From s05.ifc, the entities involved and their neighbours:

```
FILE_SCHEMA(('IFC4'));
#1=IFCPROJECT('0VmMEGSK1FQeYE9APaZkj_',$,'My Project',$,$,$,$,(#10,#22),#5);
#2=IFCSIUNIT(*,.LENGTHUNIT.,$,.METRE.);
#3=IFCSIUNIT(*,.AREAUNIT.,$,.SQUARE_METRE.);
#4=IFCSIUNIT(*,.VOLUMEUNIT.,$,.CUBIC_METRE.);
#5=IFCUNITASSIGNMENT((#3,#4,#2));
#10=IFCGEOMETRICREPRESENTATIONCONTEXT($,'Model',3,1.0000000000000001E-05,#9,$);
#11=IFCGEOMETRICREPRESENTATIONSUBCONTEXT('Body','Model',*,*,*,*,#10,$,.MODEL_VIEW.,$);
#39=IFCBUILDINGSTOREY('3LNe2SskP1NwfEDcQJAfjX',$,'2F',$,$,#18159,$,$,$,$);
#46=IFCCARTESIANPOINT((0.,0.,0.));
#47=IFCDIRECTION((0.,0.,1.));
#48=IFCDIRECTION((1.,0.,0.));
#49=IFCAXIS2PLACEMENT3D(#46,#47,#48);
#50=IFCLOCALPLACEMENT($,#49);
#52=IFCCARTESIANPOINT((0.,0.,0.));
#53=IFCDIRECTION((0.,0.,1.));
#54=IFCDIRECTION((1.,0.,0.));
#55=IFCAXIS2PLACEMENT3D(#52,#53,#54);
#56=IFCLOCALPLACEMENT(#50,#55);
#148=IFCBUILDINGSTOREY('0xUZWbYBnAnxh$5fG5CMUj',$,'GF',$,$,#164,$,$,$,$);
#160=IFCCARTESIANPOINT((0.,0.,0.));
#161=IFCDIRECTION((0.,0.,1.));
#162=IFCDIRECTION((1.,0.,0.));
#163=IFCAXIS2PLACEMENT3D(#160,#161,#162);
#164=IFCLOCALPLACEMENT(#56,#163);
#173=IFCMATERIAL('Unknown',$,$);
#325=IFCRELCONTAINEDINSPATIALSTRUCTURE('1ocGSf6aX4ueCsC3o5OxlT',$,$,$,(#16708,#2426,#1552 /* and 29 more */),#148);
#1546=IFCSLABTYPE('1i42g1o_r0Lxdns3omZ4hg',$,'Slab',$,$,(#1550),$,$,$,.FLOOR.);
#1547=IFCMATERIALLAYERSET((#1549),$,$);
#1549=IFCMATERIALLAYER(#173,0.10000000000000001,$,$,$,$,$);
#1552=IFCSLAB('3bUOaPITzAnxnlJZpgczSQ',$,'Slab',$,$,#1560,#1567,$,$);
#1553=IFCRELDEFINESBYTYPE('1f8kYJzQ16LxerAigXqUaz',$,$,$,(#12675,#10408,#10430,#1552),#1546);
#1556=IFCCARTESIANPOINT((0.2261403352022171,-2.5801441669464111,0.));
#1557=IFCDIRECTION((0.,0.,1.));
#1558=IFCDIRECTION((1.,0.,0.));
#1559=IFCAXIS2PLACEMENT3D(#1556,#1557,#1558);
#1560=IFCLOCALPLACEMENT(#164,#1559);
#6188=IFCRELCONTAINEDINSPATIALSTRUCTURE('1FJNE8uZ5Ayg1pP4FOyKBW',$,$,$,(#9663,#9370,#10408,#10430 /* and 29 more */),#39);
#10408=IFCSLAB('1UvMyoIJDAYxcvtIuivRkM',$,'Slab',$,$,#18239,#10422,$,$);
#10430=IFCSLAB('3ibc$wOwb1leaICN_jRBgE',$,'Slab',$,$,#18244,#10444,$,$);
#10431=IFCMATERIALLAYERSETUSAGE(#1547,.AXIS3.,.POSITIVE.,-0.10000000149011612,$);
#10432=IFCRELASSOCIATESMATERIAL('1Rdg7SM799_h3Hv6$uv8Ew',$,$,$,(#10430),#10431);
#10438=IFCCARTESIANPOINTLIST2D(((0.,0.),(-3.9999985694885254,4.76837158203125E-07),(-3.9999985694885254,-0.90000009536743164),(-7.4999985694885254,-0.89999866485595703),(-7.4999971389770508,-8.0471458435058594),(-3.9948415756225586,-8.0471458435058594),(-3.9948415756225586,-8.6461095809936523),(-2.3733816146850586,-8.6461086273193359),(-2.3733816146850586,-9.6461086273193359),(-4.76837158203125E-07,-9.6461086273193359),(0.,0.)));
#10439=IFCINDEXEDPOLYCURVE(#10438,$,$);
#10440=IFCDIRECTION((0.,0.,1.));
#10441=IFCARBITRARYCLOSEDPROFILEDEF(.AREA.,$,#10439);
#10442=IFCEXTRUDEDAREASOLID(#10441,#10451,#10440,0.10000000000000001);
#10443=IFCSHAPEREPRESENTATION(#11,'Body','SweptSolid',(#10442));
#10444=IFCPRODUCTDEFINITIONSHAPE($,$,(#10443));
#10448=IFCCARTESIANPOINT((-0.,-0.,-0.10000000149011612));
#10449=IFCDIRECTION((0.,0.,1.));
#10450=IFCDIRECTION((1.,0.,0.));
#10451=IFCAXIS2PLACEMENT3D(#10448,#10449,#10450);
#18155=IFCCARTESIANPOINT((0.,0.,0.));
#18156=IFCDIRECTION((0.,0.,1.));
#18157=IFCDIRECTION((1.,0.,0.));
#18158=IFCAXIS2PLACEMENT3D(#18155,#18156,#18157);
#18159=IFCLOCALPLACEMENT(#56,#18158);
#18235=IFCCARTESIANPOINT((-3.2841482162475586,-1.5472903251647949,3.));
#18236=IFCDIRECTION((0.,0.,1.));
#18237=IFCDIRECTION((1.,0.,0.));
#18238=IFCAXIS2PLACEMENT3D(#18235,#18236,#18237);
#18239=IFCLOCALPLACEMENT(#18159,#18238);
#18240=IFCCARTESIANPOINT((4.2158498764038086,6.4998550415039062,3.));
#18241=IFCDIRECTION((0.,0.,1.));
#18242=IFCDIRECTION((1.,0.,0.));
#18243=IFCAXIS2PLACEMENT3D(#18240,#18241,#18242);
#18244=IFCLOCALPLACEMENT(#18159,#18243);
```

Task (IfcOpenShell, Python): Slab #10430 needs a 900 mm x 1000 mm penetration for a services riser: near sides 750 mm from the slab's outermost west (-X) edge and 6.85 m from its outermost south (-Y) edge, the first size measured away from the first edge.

```python
import numpy as np
import ifcopenshell
import ifcopenshell.api.feature
import ifcopenshell.api.geometry
import ifcopenshell.api.root
import ifcopenshell.geom
import ifcopenshell.util.placement
import ifcopenshell.util.representation
import ifcopenshell.util.shape
import ifcopenshell.util.unit

model = ifcopenshell.open("s05.ifc")
unit_scale = ifcopenshell.util.unit.calculate_unit_scale(model)
settings = ifcopenshell.geom.settings()


def volume(element):
    """Net volume in cubic metres, openings subtracted."""
    shape = ifcopenshell.geom.create_shape(settings, element)
    return ifcopenshell.util.shape.get_volume(shape.geometry)


slab = model.by_guid("3ibc$wOwb1leaICN_jRBgE")
before = volume(slab)

# Extent in the slab's own axes, in metres. The edges named are its -X and -Y sides.
slab_shape = ifcopenshell.geom.create_shape(settings, slab)
vertices = ifcopenshell.util.shape.get_vertices(slab_shape.geometry)
x_min, y_min, bottom = vertices.min(axis=0)
top = vertices[:, 2].max()

opening = ifcopenshell.api.root.create_entity(model, ifc_class="IfcOpeningElement", name="Services riser opening", predefined_type="OPENING")
context = ifcopenshell.util.representation.get_context(model, "Model", "Body", "MODEL_VIEW")
width, depth = 0.9, 1
outline = [(0.0, 0.0), (width, 0.0), (width, depth), (0.0, depth), (0.0, 0.0)]
# Overshoot both faces by 50 mm so the cut is clean.
shape = ifcopenshell.api.geometry.add_slab_representation(
    model, context=context, depth=top - bottom + 0.1, polyline=outline
)
ifcopenshell.api.geometry.assign_representation(model, product=opening, representation=shape)

matrix = ifcopenshell.util.placement.get_local_placement(slab.ObjectPlacement)
matrix[:, 3] = matrix @ np.append(np.array([x_min + 0.75, y_min + 6.85, bottom - 0.05]) / unit_scale, 1.0)
ifcopenshell.api.geometry.edit_object_placement(model, product=opening, matrix=matrix, is_si=False)
ifcopenshell.api.feature.add_feature(model, feature=opening, element=slab)

after = volume(slab)

print(f"slab volume {before:.3f} -> {after:.3f} m3")

model.write("s05_rev.ifc")
```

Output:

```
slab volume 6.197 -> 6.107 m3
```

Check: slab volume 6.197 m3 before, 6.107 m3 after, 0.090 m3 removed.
